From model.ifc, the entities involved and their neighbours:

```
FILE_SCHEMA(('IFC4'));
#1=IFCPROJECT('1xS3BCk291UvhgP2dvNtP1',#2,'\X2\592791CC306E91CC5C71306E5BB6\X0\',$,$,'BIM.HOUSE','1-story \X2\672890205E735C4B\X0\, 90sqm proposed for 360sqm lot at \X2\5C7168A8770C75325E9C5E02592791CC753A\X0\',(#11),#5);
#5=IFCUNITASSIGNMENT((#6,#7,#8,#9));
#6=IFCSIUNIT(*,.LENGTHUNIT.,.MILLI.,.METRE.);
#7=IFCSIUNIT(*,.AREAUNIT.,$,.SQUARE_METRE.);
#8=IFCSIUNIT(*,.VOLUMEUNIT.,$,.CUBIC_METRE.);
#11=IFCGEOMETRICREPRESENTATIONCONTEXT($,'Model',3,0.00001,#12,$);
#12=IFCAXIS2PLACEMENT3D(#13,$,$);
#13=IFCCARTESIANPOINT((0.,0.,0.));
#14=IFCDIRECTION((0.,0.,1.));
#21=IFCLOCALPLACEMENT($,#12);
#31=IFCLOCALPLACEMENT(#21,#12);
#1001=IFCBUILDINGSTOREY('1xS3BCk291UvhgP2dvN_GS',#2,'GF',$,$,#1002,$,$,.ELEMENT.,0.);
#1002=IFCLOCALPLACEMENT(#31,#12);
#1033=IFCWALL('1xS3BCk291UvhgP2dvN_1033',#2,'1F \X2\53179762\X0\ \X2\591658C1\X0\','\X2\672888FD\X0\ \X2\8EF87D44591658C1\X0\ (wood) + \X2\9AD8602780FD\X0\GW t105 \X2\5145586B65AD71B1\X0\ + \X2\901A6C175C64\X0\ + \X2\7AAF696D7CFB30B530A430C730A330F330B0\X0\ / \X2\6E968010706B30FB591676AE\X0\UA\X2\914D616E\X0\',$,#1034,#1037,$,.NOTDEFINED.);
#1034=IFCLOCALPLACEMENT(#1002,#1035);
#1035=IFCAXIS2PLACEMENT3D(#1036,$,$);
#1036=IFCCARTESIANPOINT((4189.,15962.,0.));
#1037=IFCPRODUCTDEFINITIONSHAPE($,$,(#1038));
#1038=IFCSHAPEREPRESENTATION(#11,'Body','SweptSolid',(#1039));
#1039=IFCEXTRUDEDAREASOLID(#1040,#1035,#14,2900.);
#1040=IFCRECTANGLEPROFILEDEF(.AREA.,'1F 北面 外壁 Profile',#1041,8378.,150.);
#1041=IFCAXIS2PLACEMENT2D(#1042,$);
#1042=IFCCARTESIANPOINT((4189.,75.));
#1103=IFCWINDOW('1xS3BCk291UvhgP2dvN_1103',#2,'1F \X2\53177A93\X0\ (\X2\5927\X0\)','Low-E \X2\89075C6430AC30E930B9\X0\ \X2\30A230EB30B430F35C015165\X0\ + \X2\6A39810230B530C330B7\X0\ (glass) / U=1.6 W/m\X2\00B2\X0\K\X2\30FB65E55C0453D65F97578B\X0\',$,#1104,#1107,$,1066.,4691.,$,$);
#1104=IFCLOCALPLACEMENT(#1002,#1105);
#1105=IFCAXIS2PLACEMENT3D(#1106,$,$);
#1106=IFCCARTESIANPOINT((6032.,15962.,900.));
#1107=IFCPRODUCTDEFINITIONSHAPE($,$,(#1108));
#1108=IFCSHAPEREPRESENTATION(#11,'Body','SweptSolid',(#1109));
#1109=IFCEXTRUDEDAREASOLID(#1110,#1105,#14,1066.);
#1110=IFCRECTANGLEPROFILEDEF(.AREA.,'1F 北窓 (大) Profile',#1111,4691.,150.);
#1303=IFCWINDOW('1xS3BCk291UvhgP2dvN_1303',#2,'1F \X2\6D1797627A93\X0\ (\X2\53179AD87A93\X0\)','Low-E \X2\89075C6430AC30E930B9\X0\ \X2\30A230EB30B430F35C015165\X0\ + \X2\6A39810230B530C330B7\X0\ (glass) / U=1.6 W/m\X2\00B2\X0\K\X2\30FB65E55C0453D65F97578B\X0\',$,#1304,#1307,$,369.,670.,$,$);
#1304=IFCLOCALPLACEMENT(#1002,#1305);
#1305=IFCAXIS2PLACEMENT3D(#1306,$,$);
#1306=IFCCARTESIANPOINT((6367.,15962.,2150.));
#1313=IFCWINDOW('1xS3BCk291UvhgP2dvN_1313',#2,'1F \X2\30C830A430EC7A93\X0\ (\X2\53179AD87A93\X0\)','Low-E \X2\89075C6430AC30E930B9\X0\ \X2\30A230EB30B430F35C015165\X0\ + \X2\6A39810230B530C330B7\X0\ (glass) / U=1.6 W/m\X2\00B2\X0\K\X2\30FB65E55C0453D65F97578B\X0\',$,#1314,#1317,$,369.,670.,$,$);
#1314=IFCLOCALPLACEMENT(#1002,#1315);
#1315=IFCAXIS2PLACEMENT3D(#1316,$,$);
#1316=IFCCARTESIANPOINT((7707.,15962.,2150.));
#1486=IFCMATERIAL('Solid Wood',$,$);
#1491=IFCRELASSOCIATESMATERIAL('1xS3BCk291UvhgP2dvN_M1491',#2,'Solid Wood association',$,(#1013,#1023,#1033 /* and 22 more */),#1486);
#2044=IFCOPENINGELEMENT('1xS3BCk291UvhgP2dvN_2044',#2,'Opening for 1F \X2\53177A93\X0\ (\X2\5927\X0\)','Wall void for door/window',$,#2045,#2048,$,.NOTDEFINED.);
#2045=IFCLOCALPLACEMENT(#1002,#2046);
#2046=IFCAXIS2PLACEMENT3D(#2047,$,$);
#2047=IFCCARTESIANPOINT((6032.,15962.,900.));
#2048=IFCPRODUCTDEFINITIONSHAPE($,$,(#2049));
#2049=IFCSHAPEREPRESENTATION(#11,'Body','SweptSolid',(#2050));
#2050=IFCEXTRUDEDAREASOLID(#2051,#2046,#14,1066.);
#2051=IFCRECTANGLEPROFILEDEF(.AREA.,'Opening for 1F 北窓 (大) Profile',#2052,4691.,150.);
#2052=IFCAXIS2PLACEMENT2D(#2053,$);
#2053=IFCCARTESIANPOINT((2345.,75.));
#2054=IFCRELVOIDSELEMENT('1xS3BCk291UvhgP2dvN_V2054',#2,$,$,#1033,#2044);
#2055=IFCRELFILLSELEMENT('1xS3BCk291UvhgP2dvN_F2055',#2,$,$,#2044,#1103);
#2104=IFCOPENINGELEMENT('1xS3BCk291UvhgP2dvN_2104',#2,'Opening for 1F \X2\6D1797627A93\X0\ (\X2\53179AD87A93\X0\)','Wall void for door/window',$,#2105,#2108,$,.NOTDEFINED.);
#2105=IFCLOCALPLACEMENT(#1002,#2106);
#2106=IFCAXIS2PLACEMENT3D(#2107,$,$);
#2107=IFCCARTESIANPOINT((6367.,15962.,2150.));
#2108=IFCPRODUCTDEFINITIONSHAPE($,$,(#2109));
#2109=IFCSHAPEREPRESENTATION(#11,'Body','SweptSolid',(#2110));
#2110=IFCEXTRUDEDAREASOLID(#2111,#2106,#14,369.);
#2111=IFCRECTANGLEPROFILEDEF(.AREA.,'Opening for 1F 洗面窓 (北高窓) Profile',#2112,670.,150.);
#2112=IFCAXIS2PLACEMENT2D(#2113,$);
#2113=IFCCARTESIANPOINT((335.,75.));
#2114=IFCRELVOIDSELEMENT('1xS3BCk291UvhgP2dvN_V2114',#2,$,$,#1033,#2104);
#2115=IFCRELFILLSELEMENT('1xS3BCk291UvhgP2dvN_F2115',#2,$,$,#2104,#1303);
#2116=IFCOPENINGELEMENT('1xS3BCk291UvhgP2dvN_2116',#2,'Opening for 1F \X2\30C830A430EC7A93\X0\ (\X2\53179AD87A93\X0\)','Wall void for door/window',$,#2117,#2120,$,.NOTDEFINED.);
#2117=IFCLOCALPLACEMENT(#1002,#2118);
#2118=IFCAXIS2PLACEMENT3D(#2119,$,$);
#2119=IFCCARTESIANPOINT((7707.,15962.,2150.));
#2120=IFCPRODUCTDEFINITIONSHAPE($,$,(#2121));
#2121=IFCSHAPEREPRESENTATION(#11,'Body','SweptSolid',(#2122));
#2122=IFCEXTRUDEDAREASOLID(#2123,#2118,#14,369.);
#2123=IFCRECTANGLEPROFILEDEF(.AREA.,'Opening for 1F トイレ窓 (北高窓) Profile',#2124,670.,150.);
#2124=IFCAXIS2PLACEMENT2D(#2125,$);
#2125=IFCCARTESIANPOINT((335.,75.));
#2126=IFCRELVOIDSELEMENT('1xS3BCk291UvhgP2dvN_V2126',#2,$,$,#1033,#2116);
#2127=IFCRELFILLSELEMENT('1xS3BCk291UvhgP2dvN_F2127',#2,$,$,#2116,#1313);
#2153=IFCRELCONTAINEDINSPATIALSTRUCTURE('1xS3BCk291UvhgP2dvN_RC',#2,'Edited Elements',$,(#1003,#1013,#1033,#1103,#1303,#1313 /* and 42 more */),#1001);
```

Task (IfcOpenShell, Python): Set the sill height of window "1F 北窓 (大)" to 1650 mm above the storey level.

```python
import numpy as np
import ifcopenshell
import ifcopenshell.api.geometry
import ifcopenshell.geom
import ifcopenshell.util.element
import ifcopenshell.util.placement
import ifcopenshell.util.shape
import ifcopenshell.util.unit

model = ifcopenshell.open("model.ifc")
unit_scale = ifcopenshell.util.unit.calculate_unit_scale(model)

window = model.by_guid("1xS3BCk291UvhgP2dvN_1103")
opening = window.FillsVoids[0].RelatingOpeningElement
storey = ifcopenshell.util.element.get_container(window, ifc_class="IfcBuildingStorey")
level = ifcopenshell.util.placement.get_local_placement(storey.ObjectPlacement)[2, 3]

# The opening's origin need not be at the sill, so measure its lowest point.
shape = ifcopenshell.geom.create_shape(ifcopenshell.geom.settings(), opening)
bottom = ifcopenshell.util.shape.get_shape_bottom_elevation(shape, shape.geometry) / unit_scale
dz = level + 1.65 / unit_scale - bottom

shift = np.array([0.0, 0.0, dz])
# The window is not placed relative to its opening, so move both.
for product in (opening, window):
    matrix = ifcopenshell.util.placement.get_local_placement(product.ObjectPlacement)
    matrix[:3, 3] += shift
    ifcopenshell.api.geometry.edit_object_placement(model, product=product, matrix=matrix, is_si=False)

print(f"moved by {dz * unit_scale:+.3f} m")

model.write("model_v2.ifc")
```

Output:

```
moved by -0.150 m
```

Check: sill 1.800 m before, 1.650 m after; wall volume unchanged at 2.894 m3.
